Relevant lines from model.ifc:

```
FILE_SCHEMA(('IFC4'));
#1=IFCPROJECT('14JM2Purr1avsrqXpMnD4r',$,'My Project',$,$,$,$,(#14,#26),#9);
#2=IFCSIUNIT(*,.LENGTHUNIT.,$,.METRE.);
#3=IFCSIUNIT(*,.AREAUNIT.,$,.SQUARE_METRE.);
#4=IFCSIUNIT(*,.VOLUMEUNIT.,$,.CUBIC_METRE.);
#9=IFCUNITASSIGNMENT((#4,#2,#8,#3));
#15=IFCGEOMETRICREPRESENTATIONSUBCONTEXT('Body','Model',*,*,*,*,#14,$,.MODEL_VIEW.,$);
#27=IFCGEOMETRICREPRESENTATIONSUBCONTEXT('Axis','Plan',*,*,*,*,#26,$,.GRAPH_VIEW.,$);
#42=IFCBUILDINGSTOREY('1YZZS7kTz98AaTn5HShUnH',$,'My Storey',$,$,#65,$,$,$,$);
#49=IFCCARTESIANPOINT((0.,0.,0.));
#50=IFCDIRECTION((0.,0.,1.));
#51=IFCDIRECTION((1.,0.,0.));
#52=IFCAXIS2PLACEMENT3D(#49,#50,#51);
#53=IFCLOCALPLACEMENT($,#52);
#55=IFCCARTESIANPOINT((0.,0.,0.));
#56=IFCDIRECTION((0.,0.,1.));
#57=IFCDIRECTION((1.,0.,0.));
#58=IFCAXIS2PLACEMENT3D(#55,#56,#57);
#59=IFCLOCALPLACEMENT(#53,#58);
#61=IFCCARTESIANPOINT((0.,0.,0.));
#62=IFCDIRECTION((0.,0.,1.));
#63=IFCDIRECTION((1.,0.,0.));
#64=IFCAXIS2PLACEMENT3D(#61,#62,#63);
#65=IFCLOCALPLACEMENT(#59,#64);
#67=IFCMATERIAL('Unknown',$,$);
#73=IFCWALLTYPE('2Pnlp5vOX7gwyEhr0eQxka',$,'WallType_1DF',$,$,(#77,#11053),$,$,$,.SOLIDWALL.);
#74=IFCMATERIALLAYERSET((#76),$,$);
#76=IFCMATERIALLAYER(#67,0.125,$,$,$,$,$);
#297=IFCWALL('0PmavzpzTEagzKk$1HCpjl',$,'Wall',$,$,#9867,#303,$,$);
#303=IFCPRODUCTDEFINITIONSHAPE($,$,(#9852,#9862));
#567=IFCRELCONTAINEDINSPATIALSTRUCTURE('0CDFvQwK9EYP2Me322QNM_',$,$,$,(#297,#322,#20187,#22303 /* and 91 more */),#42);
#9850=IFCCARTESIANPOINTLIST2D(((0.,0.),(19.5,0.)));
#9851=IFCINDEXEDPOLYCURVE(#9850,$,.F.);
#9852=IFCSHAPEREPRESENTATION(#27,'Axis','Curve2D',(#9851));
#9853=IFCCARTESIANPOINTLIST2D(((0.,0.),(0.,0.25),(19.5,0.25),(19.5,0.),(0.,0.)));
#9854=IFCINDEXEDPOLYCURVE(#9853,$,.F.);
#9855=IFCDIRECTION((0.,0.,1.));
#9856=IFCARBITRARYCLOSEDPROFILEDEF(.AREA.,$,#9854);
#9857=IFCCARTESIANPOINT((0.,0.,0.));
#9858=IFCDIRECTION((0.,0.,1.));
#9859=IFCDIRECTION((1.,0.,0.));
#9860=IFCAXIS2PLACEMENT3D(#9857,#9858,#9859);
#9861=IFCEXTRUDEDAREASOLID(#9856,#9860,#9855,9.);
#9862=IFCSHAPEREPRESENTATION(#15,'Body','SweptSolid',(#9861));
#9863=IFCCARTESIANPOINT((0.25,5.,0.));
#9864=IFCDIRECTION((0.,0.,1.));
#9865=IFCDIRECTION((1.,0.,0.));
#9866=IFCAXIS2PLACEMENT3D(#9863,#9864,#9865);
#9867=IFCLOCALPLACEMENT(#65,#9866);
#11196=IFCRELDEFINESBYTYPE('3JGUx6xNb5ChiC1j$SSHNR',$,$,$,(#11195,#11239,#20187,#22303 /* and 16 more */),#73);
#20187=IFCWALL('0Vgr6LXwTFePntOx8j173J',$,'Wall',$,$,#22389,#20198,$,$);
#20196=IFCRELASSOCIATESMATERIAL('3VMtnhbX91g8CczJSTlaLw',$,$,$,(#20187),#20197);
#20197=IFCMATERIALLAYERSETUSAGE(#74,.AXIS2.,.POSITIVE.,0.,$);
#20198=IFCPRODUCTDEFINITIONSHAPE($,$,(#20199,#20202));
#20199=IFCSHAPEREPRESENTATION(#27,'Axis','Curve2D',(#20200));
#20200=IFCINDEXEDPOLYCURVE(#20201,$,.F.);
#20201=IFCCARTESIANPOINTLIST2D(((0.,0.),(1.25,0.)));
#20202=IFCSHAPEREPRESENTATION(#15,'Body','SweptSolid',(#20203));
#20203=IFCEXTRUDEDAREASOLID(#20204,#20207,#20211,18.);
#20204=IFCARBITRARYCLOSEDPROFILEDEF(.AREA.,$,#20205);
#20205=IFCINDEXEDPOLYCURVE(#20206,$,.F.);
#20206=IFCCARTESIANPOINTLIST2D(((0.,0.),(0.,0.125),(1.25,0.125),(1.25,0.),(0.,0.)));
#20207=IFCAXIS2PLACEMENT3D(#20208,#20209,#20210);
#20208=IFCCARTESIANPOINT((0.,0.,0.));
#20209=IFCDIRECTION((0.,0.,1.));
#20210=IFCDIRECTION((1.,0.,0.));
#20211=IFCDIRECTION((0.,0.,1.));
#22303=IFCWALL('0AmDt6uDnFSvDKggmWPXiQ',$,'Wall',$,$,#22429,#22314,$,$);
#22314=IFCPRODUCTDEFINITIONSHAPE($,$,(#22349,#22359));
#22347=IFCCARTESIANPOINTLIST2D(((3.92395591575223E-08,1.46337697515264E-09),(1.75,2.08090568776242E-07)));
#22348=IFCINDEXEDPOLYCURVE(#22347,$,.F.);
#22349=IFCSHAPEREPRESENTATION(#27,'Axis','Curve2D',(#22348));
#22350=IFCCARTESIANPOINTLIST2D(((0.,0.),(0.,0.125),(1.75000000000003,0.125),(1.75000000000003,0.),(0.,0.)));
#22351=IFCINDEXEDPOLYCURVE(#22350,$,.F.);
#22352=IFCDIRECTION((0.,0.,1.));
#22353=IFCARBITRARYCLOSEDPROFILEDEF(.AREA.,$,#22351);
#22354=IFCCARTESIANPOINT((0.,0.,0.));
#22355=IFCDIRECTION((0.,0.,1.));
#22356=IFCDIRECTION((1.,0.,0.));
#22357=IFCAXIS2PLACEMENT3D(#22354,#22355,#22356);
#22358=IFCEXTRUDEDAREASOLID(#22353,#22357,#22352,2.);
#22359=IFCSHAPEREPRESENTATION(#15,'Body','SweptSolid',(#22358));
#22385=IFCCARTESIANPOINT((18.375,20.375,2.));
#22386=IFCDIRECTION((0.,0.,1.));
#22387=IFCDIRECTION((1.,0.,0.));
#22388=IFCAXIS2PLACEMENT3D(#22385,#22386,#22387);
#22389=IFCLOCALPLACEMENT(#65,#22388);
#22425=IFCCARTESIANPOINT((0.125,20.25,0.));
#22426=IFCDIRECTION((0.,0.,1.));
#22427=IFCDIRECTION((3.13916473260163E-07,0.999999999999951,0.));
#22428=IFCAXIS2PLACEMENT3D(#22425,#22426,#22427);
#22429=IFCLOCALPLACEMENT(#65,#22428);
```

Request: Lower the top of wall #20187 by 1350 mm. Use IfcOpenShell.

```python
import ifcopenshell
import ifcopenshell.geom
import ifcopenshell.util.representation
import ifcopenshell.util.shape
import ifcopenshell.util.unit

model = ifcopenshell.open("model.ifc")
unit_scale = ifcopenshell.util.unit.calculate_unit_scale(model)
settings = ifcopenshell.geom.settings()


def volume(element):
    """Net volume in cubic metres, openings subtracted."""
    shape = ifcopenshell.geom.create_shape(settings, element)
    return ifcopenshell.util.shape.get_volume(shape.geometry)


wall = model.by_guid("0Vgr6LXwTFePntOx8j173J")
before = volume(wall)

body = ifcopenshell.util.representation.get_representation(wall, "Model", "Body")
solid = body.Items[0]
old_height = solid.Depth
solid.Depth -= 1.35 / unit_scale
after = volume(wall)

print(f"height {old_height:g} -> {solid.Depth:g}, volume {before:.3f} -> {after:.3f} m3")

model.write("model_rev.ifc")
```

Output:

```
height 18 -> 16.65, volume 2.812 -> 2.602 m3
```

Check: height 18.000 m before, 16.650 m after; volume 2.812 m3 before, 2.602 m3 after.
